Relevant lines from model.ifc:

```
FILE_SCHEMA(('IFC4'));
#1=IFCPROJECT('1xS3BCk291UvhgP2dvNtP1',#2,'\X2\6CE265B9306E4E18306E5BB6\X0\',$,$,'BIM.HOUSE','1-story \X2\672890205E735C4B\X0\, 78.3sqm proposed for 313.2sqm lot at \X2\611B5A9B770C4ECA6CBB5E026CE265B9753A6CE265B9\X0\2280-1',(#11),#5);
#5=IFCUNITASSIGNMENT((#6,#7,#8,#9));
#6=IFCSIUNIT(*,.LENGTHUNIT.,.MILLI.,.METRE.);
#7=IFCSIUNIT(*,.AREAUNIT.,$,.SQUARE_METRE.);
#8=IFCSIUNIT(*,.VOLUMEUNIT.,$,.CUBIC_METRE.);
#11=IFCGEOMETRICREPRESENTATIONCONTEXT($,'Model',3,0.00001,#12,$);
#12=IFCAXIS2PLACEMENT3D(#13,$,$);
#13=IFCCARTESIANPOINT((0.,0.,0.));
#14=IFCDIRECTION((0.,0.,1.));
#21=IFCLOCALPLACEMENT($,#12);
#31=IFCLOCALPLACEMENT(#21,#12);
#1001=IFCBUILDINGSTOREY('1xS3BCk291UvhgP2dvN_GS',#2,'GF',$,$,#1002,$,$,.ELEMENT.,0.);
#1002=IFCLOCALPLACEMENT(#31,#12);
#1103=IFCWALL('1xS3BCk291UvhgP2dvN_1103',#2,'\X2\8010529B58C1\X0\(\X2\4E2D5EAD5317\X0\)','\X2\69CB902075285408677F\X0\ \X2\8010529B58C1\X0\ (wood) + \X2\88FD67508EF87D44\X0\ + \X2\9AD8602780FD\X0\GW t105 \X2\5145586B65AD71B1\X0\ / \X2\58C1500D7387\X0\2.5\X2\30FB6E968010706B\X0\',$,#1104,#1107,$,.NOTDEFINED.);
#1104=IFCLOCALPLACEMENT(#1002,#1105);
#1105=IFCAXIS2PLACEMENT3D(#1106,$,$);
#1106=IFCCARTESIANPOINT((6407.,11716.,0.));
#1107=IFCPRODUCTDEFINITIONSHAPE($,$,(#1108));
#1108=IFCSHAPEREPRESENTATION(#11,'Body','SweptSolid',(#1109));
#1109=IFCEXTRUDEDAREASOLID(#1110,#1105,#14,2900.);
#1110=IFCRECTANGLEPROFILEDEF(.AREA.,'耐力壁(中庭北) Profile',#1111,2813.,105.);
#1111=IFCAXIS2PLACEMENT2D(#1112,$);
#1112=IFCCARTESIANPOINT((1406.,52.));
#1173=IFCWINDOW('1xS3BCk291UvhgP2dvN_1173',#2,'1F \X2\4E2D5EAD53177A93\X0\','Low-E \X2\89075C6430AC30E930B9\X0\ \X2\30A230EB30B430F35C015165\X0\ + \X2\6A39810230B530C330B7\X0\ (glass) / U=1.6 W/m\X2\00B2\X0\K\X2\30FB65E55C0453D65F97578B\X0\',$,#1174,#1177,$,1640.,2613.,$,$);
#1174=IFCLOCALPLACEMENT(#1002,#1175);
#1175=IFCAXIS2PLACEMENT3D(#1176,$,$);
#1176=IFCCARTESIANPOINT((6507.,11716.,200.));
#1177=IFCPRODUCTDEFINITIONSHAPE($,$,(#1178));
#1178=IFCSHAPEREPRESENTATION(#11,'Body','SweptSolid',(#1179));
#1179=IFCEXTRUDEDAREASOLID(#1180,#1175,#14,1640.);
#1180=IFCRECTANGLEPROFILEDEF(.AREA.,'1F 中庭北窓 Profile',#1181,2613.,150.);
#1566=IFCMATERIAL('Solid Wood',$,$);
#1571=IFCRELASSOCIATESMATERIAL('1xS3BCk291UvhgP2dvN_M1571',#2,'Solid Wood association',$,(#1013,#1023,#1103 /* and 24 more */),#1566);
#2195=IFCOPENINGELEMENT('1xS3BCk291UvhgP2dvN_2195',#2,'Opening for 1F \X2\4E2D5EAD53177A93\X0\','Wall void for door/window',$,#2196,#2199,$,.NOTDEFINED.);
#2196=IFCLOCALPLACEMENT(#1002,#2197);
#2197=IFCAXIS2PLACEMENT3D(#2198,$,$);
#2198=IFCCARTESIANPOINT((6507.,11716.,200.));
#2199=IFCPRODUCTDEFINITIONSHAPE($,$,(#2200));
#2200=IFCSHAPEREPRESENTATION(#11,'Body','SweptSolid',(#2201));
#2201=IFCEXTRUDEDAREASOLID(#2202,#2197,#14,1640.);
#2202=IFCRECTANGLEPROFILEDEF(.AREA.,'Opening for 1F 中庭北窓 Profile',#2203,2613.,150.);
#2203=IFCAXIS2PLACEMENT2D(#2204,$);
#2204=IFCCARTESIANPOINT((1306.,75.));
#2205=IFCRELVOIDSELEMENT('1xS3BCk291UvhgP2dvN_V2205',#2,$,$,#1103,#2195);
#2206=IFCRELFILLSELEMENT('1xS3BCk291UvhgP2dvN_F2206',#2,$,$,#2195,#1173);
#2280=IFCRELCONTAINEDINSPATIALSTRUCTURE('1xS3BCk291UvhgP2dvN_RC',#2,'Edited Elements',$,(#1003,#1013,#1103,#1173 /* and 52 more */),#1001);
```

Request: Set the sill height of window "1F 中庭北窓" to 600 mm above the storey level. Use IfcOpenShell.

```python
import numpy as np
import ifcopenshell
import ifcopenshell.api.geometry
import ifcopenshell.geom
import ifcopenshell.util.element
import ifcopenshell.util.placement
import ifcopenshell.util.shape
import ifcopenshell.util.unit

model = ifcopenshell.open("model.ifc")
unit_scale = ifcopenshell.util.unit.calculate_unit_scale(model)

window = model.by_guid("1xS3BCk291UvhgP2dvN_1173")
opening = window.FillsVoids[0].RelatingOpeningElement
storey = ifcopenshell.util.element.get_container(window, ifc_class="IfcBuildingStorey")
level = ifcopenshell.util.placement.get_local_placement(storey.ObjectPlacement)[2, 3]

# The opening's origin need not be at the sill, so measure its lowest point.
shape = ifcopenshell.geom.create_shape(ifcopenshell.geom.settings(), opening)
bottom = ifcopenshell.util.shape.get_shape_bottom_elevation(shape, shape.geometry) / unit_scale
dz = level + 0.6 / unit_scale - bottom

shift = np.array([0.0, 0.0, dz])
# The window is not placed relative to its opening, so move both.
for product in (opening, window):
    matrix = ifcopenshell.util.placement.get_local_placement(product.ObjectPlacement)
    matrix[:3, 3] += shift
    ifcopenshell.api.geometry.edit_object_placement(model, product=product, matrix=matrix, is_si=False)

print(f"moved by {dz * unit_scale:+.3f} m")

model.write("model_edited.ifc")
```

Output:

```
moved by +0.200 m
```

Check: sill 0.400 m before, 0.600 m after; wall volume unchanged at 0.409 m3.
